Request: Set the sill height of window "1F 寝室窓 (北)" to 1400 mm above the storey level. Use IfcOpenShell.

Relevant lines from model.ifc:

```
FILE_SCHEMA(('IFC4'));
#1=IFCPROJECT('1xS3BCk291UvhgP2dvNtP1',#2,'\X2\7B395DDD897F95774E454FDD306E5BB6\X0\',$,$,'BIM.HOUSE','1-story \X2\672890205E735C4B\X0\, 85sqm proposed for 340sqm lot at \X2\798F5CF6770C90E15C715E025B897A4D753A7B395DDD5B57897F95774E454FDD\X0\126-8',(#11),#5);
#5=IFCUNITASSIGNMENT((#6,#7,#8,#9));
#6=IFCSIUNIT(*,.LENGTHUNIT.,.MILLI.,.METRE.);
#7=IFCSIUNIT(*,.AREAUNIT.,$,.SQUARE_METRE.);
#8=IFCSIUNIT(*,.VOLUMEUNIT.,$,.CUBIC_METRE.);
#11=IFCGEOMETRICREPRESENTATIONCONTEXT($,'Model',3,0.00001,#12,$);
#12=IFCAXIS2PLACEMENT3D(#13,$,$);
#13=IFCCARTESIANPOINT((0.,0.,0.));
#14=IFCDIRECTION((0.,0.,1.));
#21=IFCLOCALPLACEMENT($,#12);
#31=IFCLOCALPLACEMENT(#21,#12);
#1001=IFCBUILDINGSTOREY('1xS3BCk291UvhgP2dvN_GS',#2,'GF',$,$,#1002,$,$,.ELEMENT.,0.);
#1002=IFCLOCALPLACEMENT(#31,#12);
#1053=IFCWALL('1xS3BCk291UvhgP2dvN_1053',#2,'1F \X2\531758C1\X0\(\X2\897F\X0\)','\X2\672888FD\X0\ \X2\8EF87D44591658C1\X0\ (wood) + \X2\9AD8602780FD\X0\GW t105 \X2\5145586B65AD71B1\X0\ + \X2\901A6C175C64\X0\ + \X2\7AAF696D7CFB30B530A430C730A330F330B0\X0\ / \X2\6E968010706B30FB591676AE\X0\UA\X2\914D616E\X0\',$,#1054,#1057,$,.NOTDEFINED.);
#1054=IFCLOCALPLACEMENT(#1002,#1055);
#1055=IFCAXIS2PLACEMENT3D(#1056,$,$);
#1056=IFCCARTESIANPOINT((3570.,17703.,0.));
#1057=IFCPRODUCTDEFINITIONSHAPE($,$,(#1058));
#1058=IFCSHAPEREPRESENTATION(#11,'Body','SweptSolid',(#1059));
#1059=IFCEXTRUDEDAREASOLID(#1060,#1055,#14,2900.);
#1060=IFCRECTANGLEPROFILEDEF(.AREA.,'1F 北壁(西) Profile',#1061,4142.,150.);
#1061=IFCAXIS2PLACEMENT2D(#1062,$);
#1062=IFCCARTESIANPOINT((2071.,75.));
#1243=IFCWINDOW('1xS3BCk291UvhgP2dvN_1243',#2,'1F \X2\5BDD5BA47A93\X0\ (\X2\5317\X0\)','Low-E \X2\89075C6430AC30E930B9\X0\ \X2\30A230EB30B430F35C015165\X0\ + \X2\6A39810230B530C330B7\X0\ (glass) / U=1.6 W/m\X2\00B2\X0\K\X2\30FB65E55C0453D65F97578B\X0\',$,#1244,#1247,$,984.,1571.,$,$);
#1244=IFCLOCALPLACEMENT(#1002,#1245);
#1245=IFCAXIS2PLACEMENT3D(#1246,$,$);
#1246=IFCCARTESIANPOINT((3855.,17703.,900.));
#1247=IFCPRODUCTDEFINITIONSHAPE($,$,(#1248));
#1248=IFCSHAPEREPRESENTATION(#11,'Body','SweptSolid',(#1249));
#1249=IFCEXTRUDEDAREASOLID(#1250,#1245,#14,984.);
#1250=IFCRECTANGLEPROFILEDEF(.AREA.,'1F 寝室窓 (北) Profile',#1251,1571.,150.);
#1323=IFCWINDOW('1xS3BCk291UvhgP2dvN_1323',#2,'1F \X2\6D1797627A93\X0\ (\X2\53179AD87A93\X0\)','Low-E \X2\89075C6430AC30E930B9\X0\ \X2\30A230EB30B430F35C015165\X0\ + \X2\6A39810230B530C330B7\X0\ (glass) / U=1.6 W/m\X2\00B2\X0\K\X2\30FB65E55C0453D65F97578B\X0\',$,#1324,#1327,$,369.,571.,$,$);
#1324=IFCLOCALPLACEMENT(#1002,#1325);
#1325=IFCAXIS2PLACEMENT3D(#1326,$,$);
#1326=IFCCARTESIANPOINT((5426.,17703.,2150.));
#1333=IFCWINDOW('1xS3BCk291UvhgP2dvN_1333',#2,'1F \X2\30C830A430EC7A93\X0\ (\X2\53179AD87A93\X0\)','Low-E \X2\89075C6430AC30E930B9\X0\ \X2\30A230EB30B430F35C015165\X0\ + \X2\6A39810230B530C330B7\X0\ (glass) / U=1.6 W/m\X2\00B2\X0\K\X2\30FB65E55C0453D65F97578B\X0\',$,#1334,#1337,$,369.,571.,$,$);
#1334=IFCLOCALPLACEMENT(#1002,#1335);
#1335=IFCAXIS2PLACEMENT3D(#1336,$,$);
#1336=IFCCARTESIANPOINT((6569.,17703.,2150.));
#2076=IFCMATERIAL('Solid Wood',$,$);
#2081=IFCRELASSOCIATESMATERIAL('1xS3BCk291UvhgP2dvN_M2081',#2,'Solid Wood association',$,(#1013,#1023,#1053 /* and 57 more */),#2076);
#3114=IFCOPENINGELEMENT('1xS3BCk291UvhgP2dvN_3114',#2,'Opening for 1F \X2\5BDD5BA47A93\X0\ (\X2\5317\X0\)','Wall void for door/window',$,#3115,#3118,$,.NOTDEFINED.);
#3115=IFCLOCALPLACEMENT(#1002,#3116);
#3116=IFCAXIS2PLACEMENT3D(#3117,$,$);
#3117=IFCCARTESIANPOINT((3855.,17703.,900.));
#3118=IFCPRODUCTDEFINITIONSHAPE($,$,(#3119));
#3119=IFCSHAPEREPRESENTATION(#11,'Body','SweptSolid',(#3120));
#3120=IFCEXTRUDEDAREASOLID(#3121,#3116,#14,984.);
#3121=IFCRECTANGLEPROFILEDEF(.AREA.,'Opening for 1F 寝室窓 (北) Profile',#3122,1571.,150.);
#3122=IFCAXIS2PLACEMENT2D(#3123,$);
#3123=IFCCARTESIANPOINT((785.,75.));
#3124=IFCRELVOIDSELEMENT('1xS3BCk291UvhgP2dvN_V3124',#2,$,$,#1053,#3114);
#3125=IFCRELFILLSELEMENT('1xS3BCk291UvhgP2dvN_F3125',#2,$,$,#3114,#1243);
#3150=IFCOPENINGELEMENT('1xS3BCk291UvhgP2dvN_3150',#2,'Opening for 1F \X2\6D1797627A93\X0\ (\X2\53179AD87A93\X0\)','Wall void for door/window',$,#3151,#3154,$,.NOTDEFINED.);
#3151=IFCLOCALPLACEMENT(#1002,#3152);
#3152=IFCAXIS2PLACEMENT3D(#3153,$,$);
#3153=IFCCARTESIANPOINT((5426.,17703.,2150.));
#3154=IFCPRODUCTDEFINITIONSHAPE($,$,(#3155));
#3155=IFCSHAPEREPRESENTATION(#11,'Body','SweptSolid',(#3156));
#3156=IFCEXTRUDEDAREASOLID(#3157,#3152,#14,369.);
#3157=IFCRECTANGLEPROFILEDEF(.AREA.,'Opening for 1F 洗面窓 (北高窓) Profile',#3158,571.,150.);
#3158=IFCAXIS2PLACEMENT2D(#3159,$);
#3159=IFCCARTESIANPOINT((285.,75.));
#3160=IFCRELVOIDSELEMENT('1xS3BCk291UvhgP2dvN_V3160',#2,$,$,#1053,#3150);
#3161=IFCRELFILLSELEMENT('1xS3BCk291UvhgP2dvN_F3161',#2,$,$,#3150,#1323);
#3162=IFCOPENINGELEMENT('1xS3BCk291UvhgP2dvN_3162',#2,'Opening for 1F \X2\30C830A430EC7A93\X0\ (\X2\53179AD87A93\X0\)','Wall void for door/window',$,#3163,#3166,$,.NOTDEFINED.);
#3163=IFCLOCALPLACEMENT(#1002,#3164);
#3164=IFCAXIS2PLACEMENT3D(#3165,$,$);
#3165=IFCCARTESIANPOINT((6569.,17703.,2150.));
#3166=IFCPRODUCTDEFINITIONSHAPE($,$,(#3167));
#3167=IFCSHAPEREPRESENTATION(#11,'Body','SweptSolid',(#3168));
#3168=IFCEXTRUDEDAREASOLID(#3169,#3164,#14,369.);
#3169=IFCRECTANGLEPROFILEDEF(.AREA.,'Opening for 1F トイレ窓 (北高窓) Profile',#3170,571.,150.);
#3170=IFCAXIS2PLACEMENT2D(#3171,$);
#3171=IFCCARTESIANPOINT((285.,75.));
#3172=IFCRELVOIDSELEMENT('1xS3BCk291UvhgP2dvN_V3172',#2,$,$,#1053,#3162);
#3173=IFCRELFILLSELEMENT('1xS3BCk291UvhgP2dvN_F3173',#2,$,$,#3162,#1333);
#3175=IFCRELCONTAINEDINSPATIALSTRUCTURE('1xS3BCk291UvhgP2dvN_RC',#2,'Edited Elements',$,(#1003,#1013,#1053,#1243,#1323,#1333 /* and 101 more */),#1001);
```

```python
import numpy as np
import ifcopenshell
import ifcopenshell.api.geometry
import ifcopenshell.geom
import ifcopenshell.util.element
import ifcopenshell.util.placement
import ifcopenshell.util.shape
import ifcopenshell.util.unit

model = ifcopenshell.open("model.ifc")
unit_scale = ifcopenshell.util.unit.calculate_unit_scale(model)

window = model.by_guid("1xS3BCk291UvhgP2dvN_1243")
opening = window.FillsVoids[0].RelatingOpeningElement
storey = ifcopenshell.util.element.get_container(window, ifc_class="IfcBuildingStorey")
level = ifcopenshell.util.placement.get_local_placement(storey.ObjectPlacement)[2, 3]

# The opening's origin need not be at the sill, so measure its lowest point.
shape = ifcopenshell.geom.create_shape(ifcopenshell.geom.settings(), opening)
bottom = ifcopenshell.util.shape.get_shape_bottom_elevation(shape, shape.geometry) / unit_scale
dz = level + 1.4 / unit_scale - bottom

shift = np.array([0.0, 0.0, dz])
# The window is not placed relative to its opening, so move both.
for product in (opening, window):
    matrix = ifcopenshell.util.placement.get_local_placement(product.ObjectPlacement)
    matrix[:3, 3] += shift
    ifcopenshell.api.geometry.edit_object_placement(model, product=product, matrix=matrix, is_si=False)

print(f"moved by {dz * unit_scale:+.3f} m")

model.write("model_edited.ifc")
```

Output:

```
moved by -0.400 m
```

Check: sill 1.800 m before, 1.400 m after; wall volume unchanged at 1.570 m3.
